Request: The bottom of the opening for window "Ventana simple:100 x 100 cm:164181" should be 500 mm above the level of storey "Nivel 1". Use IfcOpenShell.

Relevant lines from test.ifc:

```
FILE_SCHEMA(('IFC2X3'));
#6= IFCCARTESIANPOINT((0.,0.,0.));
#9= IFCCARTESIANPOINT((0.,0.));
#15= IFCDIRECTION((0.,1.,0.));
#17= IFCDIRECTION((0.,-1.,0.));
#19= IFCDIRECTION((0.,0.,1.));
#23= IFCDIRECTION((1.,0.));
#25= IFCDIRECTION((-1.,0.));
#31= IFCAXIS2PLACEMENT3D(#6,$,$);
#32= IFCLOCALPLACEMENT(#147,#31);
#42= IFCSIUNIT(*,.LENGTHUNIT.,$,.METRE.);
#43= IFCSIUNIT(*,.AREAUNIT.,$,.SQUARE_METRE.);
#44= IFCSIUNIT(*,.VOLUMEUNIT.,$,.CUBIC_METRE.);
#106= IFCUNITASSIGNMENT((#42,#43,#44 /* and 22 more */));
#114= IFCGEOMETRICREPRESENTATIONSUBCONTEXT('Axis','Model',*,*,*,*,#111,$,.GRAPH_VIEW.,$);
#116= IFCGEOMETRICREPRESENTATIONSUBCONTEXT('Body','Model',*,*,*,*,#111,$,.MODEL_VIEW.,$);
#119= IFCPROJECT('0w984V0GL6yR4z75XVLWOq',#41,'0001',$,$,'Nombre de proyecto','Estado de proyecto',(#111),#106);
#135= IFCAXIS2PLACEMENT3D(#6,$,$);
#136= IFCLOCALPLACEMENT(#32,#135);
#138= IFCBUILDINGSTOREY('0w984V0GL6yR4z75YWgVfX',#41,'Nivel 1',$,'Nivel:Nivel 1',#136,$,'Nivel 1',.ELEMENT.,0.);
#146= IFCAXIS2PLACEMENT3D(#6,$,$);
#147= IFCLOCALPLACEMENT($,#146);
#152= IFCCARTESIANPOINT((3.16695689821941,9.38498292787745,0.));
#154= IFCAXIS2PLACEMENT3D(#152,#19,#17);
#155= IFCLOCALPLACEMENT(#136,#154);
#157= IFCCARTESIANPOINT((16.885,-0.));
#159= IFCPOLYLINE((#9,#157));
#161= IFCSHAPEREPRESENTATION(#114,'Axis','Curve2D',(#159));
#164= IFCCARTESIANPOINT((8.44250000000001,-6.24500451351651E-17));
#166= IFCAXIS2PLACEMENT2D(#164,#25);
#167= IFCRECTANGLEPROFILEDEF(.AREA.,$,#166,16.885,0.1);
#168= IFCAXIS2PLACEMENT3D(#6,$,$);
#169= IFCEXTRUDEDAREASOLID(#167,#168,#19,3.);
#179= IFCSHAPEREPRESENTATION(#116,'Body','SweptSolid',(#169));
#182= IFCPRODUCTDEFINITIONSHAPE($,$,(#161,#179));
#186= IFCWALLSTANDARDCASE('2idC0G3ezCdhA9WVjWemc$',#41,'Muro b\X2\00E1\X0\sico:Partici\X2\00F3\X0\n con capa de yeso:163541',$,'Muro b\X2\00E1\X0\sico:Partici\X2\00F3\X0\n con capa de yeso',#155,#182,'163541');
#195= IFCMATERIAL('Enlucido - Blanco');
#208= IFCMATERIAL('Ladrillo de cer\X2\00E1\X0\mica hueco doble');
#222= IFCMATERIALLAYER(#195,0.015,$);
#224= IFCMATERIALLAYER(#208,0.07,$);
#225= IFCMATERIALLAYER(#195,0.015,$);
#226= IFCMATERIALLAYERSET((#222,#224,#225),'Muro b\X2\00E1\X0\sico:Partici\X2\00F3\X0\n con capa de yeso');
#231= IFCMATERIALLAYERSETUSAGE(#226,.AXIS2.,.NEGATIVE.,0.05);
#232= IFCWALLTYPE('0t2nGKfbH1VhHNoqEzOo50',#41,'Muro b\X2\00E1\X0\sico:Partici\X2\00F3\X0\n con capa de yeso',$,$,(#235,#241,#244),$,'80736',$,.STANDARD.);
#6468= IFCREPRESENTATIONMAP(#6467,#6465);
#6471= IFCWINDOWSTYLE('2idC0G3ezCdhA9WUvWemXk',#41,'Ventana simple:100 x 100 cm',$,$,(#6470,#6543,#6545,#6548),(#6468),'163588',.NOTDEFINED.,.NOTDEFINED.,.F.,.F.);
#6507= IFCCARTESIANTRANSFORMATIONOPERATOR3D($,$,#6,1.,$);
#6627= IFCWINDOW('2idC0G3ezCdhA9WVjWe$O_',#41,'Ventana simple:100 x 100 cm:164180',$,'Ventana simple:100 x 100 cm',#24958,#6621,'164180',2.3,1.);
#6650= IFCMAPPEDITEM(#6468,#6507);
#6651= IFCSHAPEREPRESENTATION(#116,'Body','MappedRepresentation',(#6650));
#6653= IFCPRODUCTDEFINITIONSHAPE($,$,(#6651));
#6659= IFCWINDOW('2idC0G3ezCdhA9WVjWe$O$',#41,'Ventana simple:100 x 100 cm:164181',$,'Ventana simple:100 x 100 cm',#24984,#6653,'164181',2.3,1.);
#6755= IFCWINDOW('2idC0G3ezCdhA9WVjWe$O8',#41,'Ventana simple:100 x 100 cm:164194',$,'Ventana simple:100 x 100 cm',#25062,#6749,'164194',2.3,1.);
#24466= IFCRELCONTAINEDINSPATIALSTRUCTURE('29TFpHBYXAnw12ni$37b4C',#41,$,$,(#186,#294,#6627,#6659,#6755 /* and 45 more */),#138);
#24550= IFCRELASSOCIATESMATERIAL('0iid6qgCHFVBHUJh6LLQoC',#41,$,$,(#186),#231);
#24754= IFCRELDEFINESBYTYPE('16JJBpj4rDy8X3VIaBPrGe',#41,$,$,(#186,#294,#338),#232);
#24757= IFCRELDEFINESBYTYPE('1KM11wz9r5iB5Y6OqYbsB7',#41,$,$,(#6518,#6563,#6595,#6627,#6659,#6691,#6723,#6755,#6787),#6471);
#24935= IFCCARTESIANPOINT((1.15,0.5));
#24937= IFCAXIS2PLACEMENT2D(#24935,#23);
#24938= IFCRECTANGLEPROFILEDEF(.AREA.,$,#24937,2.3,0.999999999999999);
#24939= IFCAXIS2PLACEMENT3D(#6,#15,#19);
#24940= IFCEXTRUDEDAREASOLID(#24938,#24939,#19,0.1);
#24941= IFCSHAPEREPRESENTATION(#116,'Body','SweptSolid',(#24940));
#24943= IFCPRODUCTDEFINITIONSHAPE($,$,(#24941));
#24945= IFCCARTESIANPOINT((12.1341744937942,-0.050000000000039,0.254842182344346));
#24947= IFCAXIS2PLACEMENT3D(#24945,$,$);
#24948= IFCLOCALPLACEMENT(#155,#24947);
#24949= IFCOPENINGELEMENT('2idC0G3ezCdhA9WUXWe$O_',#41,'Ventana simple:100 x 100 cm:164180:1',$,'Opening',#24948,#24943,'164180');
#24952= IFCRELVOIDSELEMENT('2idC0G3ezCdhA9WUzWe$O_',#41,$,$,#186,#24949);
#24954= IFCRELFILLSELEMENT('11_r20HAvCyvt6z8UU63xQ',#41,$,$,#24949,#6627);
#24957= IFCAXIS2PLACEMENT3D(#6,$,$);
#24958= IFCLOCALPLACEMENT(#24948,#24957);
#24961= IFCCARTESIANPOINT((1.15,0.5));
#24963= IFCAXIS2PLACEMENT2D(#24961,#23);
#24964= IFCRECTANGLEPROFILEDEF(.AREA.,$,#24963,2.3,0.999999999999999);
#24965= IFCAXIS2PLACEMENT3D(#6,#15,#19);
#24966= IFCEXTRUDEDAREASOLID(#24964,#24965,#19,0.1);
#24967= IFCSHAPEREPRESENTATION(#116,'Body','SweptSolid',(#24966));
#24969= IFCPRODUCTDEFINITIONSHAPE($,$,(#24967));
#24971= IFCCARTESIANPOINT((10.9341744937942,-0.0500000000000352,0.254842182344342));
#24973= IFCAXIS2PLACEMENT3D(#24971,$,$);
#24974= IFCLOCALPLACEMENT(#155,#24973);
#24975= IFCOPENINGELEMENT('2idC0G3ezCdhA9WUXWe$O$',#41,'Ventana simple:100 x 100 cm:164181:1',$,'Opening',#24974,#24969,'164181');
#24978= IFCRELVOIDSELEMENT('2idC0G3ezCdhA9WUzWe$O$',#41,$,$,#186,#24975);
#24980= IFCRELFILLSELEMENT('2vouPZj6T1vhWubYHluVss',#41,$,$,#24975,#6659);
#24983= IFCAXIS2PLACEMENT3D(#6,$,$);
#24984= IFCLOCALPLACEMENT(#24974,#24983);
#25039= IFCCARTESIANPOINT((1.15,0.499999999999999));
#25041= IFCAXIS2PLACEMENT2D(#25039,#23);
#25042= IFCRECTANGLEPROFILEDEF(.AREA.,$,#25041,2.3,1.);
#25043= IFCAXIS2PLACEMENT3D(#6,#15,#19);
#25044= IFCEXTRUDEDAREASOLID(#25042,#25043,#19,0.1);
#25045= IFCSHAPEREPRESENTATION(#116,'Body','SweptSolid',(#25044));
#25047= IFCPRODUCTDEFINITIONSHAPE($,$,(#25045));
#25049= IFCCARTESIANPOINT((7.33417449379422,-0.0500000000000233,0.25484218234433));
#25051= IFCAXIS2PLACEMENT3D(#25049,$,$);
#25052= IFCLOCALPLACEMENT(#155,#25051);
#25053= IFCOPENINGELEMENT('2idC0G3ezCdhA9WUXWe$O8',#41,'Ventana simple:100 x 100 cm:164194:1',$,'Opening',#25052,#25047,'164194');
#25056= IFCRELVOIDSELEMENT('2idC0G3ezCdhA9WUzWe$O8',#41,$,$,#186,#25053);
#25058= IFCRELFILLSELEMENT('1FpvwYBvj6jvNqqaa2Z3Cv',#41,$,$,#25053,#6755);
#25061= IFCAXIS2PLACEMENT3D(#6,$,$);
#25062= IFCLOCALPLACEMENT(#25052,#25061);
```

```python
import numpy as np
import ifcopenshell
import ifcopenshell.api.geometry
import ifcopenshell.geom
import ifcopenshell.util.element
import ifcopenshell.util.placement
import ifcopenshell.util.shape
import ifcopenshell.util.unit

model = ifcopenshell.open("test.ifc")
unit_scale = ifcopenshell.util.unit.calculate_unit_scale(model)

window = model.by_id(6659)
opening = window.FillsVoids[0].RelatingOpeningElement
storey = ifcopenshell.util.element.get_container(window, ifc_class="IfcBuildingStorey")
level = ifcopenshell.util.placement.get_local_placement(storey.ObjectPlacement)[2, 3]

# The opening's origin need not be at the sill, so measure its lowest point.
shape = ifcopenshell.geom.create_shape(ifcopenshell.geom.settings(), opening)
bottom = ifcopenshell.util.shape.get_shape_bottom_elevation(shape, shape.geometry) / unit_scale
dz = level + 0.5 / unit_scale - bottom

shift = np.array([0.0, 0.0, dz])
# The window is placed relative to its opening, so it follows when the opening moves.
matrix = ifcopenshell.util.placement.get_local_placement(opening.ObjectPlacement)
matrix[:3, 3] += shift
ifcopenshell.api.geometry.edit_object_placement(
    model, product=opening, matrix=matrix, is_si=False, should_transform_children=True
)

print(f"moved by {dz * unit_scale:+.3f} m")

model.write("test_edited.ifc")
```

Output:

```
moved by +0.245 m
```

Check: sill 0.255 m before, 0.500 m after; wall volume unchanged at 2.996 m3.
